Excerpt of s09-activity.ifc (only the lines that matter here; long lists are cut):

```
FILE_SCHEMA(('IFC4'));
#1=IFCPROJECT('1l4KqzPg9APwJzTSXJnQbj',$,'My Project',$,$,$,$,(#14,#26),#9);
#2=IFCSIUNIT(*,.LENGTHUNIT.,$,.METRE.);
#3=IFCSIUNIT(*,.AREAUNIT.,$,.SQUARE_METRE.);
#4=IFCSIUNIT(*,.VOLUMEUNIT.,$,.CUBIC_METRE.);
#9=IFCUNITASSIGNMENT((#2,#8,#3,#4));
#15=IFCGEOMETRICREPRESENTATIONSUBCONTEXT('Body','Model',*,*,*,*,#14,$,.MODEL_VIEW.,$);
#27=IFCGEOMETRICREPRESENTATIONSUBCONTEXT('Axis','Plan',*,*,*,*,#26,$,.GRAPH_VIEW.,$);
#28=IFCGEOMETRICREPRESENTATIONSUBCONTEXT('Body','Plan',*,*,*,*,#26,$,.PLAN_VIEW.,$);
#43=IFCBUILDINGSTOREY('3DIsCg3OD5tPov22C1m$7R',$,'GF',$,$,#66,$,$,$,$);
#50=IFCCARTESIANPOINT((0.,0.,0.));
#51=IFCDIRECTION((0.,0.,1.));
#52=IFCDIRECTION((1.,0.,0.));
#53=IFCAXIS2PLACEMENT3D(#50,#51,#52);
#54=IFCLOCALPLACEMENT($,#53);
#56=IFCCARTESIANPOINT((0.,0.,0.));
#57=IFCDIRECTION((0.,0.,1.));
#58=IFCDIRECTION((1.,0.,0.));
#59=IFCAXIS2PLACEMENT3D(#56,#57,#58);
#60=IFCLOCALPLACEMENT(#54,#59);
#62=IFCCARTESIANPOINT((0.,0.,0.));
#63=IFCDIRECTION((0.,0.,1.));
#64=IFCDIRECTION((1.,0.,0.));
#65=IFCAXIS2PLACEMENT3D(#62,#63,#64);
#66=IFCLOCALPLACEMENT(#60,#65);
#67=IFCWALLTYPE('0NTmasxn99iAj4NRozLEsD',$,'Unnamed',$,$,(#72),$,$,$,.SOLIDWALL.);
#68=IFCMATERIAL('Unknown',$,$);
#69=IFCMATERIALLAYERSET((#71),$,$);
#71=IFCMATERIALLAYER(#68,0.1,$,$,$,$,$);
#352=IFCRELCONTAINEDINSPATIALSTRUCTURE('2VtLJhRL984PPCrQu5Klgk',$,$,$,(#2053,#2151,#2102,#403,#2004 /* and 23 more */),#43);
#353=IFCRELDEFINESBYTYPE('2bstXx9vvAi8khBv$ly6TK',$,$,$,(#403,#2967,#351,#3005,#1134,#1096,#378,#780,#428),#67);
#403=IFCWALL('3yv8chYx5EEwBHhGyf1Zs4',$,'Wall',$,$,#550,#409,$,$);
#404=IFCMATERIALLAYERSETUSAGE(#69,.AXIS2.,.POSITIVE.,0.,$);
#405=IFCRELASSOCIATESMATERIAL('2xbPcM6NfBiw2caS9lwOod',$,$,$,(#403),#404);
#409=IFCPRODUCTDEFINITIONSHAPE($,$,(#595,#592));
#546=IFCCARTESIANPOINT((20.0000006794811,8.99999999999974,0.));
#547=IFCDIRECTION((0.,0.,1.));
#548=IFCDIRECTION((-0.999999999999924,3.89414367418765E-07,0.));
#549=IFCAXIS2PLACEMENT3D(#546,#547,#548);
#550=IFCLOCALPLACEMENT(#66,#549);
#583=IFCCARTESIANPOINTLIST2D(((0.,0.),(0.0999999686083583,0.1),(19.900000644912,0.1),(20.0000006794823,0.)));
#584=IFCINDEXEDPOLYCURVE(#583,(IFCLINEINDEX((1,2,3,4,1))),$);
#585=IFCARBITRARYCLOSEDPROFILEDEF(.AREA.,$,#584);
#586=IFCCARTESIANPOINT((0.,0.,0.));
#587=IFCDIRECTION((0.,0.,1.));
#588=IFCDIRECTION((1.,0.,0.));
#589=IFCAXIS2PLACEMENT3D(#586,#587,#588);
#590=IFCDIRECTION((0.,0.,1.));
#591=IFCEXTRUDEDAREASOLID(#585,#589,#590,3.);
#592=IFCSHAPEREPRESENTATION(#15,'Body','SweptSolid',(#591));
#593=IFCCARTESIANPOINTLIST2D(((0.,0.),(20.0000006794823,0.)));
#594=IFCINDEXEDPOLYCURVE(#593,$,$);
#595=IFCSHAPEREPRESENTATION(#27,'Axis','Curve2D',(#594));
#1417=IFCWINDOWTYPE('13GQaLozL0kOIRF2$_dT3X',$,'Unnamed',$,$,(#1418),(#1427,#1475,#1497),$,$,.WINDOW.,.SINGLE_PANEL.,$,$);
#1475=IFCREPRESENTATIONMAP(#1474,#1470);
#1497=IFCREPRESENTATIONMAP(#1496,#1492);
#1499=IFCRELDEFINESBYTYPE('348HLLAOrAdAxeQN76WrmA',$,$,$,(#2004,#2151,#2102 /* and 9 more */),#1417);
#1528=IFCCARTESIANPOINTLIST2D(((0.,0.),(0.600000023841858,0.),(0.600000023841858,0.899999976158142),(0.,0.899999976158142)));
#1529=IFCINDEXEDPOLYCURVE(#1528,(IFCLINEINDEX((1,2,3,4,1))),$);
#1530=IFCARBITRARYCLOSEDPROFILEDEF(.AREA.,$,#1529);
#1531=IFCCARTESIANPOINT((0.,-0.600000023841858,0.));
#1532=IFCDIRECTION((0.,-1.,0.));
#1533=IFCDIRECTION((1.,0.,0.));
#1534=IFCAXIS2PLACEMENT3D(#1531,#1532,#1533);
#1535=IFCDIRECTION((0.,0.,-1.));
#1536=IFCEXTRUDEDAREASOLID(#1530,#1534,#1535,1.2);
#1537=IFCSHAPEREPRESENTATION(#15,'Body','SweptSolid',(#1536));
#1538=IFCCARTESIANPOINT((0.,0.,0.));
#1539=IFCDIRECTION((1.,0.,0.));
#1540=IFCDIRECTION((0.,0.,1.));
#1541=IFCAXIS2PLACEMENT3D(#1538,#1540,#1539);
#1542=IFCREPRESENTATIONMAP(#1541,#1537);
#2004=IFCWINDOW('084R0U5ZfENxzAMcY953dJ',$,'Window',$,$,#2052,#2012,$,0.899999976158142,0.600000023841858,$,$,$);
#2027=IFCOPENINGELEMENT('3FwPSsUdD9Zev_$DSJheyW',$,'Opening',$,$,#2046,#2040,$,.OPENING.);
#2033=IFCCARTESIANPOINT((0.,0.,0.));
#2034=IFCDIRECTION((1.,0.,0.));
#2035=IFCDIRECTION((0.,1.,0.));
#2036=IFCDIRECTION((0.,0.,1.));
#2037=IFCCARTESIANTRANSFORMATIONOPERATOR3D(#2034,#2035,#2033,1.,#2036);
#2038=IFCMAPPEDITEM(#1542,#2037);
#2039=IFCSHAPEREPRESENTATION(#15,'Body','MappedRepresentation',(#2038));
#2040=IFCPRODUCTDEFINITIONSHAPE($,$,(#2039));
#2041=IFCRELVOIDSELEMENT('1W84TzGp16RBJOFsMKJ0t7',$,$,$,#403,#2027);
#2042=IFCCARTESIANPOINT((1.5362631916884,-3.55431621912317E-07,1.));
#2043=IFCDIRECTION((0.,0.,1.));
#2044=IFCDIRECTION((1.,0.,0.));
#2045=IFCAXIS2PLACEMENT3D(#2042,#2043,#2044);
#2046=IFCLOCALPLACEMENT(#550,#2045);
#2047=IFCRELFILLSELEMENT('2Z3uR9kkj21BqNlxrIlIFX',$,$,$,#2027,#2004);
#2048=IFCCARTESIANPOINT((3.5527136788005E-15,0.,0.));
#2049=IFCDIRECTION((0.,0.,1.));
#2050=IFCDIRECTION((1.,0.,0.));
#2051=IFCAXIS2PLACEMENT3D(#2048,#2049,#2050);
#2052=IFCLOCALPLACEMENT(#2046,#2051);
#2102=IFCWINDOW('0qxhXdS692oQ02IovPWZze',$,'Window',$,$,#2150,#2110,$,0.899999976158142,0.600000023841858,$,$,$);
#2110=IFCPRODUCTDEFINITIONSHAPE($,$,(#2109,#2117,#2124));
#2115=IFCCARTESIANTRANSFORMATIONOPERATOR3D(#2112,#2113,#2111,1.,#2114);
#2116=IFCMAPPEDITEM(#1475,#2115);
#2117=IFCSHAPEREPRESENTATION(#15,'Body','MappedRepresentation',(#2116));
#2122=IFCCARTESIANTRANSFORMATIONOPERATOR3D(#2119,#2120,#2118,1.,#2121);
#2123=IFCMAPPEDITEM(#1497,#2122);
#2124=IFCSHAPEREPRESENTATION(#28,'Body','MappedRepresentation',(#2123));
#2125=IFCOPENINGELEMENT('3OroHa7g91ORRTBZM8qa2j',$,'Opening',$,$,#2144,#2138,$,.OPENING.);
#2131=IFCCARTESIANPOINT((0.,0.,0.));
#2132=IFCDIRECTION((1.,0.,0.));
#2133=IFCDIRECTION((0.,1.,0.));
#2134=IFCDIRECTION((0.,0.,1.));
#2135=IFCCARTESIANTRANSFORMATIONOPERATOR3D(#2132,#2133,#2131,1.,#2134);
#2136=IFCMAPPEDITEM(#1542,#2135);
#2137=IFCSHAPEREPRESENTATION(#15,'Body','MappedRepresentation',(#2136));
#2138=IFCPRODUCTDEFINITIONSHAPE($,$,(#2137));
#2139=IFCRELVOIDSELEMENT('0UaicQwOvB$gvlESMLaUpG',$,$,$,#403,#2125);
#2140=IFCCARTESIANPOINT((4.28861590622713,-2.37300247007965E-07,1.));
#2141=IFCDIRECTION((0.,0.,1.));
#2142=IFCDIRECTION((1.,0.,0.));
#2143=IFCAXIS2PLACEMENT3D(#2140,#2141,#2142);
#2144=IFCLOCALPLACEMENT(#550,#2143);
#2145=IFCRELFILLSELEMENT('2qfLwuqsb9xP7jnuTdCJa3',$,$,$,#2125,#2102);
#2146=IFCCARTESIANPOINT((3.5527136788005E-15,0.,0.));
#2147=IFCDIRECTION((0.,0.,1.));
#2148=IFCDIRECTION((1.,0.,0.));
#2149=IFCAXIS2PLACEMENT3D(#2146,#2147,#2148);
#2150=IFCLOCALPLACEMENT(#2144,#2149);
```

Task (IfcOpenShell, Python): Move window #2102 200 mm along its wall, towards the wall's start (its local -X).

```python
import ifcopenshell
import ifcopenshell.api.geometry
import ifcopenshell.util.placement
import ifcopenshell.util.unit

model = ifcopenshell.open("s09-activity.ifc")
unit_scale = ifcopenshell.util.unit.calculate_unit_scale(model)

window = model.by_guid("0qxhXdS692oQ02IovPWZze")
opening = window.FillsVoids[0].RelatingOpeningElement
wall = opening.VoidsElements[0].RelatingBuildingElement

wall_matrix = ifcopenshell.util.placement.get_local_placement(wall.ObjectPlacement)
shift = wall_matrix[:3, 0] * -0.2 / unit_scale
before = ifcopenshell.util.placement.get_local_placement(window.ObjectPlacement)[:3, 3].copy()

# The window is placed relative to its opening, so it follows when the opening moves.
matrix = ifcopenshell.util.placement.get_local_placement(opening.ObjectPlacement)
matrix[:3, 3] += shift
ifcopenshell.api.geometry.edit_object_placement(
    model, product=opening, matrix=matrix, is_si=False, should_transform_children=True
)

after = ifcopenshell.util.placement.get_local_placement(window.ObjectPlacement)[:3, 3]
print("window moved by", (after - before).round(3) + 0.0)

model.write("s09-activity-out.ifc")
```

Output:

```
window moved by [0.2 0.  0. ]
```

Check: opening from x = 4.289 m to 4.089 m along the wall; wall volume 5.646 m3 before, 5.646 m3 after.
